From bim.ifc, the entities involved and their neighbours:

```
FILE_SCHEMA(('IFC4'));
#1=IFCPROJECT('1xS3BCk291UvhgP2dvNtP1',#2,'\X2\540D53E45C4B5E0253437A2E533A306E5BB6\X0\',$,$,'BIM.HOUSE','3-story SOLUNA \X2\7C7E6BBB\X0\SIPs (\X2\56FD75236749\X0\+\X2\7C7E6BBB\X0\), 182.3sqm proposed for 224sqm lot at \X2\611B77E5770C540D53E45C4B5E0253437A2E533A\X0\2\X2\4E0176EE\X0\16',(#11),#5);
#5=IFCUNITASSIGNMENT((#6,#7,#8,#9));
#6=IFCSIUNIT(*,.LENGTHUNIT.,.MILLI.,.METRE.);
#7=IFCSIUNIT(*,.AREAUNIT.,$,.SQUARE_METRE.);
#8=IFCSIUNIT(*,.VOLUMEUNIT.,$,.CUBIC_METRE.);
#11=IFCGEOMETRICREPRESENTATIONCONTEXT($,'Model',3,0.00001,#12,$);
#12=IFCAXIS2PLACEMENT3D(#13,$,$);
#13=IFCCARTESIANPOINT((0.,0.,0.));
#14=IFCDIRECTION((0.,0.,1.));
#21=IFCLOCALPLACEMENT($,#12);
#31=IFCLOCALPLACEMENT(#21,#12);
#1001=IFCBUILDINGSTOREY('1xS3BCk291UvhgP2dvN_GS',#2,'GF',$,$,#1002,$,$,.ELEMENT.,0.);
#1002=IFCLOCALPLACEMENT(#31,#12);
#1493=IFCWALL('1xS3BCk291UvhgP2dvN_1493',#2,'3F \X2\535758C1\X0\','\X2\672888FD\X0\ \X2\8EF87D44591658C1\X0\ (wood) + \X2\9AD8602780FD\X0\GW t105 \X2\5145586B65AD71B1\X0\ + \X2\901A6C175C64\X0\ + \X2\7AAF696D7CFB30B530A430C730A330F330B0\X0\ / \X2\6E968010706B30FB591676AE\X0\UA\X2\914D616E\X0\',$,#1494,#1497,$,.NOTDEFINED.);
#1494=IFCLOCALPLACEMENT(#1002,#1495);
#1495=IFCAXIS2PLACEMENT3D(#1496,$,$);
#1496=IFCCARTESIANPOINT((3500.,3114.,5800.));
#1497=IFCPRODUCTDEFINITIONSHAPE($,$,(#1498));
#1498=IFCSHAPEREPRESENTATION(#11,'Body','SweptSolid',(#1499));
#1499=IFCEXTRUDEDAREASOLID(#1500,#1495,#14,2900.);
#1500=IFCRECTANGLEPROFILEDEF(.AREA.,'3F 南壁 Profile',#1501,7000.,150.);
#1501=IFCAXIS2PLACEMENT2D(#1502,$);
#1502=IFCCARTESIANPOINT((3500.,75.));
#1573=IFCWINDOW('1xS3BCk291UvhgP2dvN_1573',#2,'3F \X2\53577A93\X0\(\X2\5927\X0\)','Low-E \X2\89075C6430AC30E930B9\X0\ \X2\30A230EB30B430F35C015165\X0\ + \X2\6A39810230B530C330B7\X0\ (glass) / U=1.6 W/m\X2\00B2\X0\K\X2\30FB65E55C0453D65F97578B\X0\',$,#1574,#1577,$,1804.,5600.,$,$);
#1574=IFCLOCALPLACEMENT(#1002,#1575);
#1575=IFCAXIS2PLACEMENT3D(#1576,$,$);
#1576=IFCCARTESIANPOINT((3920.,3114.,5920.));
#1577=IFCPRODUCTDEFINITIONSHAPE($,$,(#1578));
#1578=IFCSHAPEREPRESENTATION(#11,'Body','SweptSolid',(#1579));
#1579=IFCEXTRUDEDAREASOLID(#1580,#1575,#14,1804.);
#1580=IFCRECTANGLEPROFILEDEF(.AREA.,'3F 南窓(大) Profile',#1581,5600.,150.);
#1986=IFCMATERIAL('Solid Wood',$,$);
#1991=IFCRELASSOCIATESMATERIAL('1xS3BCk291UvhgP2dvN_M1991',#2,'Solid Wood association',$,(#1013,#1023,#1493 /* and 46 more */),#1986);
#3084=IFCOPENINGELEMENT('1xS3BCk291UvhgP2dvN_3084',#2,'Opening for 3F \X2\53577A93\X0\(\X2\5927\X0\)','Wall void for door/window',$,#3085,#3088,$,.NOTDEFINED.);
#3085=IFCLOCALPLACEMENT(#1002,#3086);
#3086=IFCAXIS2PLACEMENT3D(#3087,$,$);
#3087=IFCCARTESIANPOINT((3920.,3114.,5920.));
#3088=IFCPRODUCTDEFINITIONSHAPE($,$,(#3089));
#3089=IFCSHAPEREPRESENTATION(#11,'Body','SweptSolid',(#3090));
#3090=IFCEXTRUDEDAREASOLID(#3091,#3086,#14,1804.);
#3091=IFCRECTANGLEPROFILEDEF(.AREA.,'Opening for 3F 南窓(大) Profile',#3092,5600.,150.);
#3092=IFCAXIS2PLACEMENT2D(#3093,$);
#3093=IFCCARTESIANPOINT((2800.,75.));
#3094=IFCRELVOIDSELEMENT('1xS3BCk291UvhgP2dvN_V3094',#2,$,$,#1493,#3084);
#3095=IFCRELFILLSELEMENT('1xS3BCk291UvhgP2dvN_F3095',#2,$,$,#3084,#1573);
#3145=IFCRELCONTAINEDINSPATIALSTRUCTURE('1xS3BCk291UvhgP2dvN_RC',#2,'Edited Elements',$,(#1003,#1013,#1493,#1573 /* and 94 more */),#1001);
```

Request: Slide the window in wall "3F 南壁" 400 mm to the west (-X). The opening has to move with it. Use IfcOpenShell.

```python
import ifcopenshell
import ifcopenshell.api.geometry
import ifcopenshell.util.placement

model = ifcopenshell.open("bim.ifc")

window = model.by_guid("1xS3BCk291UvhgP2dvN_1573")
opening = window.FillsVoids[0].RelatingOpeningElement
wall = opening.VoidsElements[0].RelatingBuildingElement

wall_matrix = ifcopenshell.util.placement.get_local_placement(wall.ObjectPlacement)
shift = wall_matrix[:3, 0] * -400.0
before = ifcopenshell.util.placement.get_local_placement(window.ObjectPlacement)[:3, 3].copy()

# The window is not placed relative to its opening, so move both.
for product in (opening, window):
    matrix = ifcopenshell.util.placement.get_local_placement(product.ObjectPlacement)
    matrix[:3, 3] += shift
    ifcopenshell.api.geometry.edit_object_placement(model, product=product, matrix=matrix, is_si=False)

after = ifcopenshell.util.placement.get_local_placement(window.ObjectPlacement)[:3, 3]
print("window moved by", (after - before).round(3) + 0.0)

model.write("bim-out.ifc")
```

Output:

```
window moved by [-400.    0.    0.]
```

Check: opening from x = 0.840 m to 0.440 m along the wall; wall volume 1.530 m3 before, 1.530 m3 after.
